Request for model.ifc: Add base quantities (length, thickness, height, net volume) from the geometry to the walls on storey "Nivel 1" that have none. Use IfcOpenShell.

First a look at what the model holds.

```python
import ifcopenshell
import ifcopenshell.util.element
import ifcopenshell.util.unit

model = ifcopenshell.open("model.ifc")
print(model.schema)
for unit_type in ("LENGTHUNIT", "AREAUNIT", "VOLUMEUNIT"):
    print(unit_type, ifcopenshell.util.unit.calculate_unit_scale(model, unit_type))
storey = next(s for s in model.by_type("IfcBuildingStorey") if s.Name == "Nivel 1")
walls = [e for e in ifcopenshell.util.element.get_decomposition(storey) if e.is_a("IfcWall")]
for e in sorted(walls, key=lambda e: e.id()):
    print(e.id(), e.is_a(), e.Name, list(ifcopenshell.util.element.get_psets(e, qtos_only=True)), sep=" | ")
```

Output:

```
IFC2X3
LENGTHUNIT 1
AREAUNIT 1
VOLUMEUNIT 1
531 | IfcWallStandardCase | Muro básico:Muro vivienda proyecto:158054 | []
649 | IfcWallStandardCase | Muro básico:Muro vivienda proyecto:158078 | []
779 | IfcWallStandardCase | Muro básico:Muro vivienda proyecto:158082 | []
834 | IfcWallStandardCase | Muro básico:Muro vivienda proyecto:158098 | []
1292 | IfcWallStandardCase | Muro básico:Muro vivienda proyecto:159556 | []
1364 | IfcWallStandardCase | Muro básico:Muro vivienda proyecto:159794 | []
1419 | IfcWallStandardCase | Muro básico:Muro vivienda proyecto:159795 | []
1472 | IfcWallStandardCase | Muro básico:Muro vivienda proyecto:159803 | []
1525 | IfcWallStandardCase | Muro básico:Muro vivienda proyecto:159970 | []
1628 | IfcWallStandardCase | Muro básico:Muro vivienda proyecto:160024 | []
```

```python
import ifcopenshell
import ifcopenshell.api.pset
import ifcopenshell.geom
import ifcopenshell.util.element
import ifcopenshell.util.shape
import ifcopenshell.util.unit

model = ifcopenshell.open("model.ifc")
unit_scale = ifcopenshell.util.unit.calculate_unit_scale(model)
volume_scale = ifcopenshell.util.unit.calculate_unit_scale(model, "VOLUMEUNIT")
settings = ifcopenshell.geom.settings()

storey = next(s for s in model.by_type("IfcBuildingStorey") if s.Name == "Nivel 1")
walls = [e for e in ifcopenshell.util.element.get_decomposition(storey) if e.is_a("IfcWall")]

for e in sorted(walls, key=lambda e: e.id()):
    if ifcopenshell.util.element.get_psets(e, qtos_only=True, should_inherit=False):
        continue
    # Geometry comes back in metres, in the element's own axes.
    shape = ifcopenshell.geom.create_shape(settings, e)
    values = {
        "Length": ifcopenshell.util.shape.get_x(shape.geometry) / unit_scale,
        "Width": ifcopenshell.util.shape.get_y(shape.geometry) / unit_scale,
        "Height": ifcopenshell.util.shape.get_z(shape.geometry) / unit_scale,
        "NetVolume": ifcopenshell.util.shape.get_volume(shape.geometry) / volume_scale,
    }
    qto = ifcopenshell.api.pset.add_qto(model, product=e, name="BaseQuantities")
    ifcopenshell.api.pset.edit_qto(model, qto=qto, properties=values)
    print(e.id(), {k: round(v, 3) for k, v in values.items()})

model.write("model_edited.ifc")
```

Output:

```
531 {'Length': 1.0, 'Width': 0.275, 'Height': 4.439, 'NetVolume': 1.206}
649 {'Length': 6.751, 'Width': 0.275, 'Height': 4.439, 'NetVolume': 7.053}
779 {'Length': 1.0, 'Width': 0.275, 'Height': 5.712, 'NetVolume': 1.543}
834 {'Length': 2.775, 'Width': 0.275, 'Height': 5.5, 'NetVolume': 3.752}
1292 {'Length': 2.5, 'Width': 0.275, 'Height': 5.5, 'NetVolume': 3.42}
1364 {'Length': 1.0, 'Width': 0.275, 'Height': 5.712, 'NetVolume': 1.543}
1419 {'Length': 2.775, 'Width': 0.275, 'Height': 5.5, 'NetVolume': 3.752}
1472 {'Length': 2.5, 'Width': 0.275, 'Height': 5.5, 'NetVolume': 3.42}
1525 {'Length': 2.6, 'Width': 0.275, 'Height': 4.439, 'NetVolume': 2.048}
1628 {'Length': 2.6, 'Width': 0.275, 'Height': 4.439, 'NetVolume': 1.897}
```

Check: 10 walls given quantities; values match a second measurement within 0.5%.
